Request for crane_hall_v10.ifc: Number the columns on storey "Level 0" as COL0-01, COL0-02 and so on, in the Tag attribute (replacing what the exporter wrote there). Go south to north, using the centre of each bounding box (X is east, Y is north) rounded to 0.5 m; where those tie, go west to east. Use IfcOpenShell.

First a look at what the model holds.

```python
import ifcopenshell
import ifcopenshell.util.element
import ifcopenshell.util.placement

model = ifcopenshell.open("crane_hall_v10.ifc")
print(model.schema)
storey = next(s for s in model.by_type("IfcBuildingStorey") if s.Name == "Level 0")
columns = [e for e in ifcopenshell.util.element.get_decomposition(storey) if e.is_a("IfcColumn")]
for e in sorted(columns, key=lambda e: e.id()):
    origin = ifcopenshell.util.placement.get_local_placement(e.ObjectPlacement)[:3, 3]
    print(e.id(), e.Tag, e.Name, origin.round(2) + 0.0, sep=" | ")
```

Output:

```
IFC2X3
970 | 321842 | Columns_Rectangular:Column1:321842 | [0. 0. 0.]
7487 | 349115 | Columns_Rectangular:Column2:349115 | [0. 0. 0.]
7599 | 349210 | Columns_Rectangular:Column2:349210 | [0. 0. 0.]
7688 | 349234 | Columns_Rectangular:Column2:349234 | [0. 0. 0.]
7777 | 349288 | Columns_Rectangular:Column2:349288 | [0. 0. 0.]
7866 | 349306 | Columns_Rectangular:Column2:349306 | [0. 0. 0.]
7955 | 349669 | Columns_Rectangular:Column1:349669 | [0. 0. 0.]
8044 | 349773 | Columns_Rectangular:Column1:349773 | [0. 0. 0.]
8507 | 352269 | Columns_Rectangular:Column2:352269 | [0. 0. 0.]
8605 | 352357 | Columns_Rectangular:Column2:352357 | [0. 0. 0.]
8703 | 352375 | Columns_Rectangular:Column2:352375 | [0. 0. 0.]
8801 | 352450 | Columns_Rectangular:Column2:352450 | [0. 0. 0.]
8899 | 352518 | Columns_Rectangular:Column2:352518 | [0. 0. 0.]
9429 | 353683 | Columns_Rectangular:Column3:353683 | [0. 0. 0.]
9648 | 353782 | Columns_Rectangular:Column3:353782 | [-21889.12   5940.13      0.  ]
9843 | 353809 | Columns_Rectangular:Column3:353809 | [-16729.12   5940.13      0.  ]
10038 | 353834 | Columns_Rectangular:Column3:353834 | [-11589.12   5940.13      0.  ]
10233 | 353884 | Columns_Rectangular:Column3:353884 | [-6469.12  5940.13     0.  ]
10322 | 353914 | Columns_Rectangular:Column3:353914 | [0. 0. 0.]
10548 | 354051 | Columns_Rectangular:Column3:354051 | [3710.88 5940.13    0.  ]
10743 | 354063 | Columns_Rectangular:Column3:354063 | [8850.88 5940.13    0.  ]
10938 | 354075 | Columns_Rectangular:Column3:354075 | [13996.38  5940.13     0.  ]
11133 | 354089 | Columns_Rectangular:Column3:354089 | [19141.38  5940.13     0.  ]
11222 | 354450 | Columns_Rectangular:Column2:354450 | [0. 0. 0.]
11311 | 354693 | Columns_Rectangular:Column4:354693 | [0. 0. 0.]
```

```python
import ifcopenshell
import ifcopenshell.geom
import ifcopenshell.util.element
import ifcopenshell.util.shape

model = ifcopenshell.open("crane_hall_v10.ifc")
settings = ifcopenshell.geom.settings()
settings.set("use-world-coords", True)


def centre(element):
    shape = ifcopenshell.geom.create_shape(settings, element)
    return ifcopenshell.util.shape.get_bbox_centroid(shape.geometry)


storey = next(s for s in model.by_type("IfcBuildingStorey") if s.Name == "Level 0")
columns = [e for e in ifcopenshell.util.element.get_decomposition(storey) if e.is_a("IfcColumn")]

# Insertion points can sit at a corner or the storey origin, so sort by the geometry (in metres).
centres = {e: centre(e) for e in columns}
columns.sort(key=lambda e: (round(centres[e][1] / 0.5), centres[e][0]))

for i, e in enumerate(columns, start=1):
    number = f"COL0-{i:02d}"
    e.Tag = number
    print(e.id(), number)

model.write("crane_hall_v10_edited.ifc")
```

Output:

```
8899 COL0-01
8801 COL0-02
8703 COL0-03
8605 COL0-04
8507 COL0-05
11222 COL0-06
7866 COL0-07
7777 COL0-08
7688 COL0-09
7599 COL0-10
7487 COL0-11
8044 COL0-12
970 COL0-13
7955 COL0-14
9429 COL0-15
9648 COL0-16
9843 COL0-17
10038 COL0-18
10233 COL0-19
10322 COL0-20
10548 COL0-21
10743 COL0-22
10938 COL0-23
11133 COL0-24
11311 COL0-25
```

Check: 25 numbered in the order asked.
